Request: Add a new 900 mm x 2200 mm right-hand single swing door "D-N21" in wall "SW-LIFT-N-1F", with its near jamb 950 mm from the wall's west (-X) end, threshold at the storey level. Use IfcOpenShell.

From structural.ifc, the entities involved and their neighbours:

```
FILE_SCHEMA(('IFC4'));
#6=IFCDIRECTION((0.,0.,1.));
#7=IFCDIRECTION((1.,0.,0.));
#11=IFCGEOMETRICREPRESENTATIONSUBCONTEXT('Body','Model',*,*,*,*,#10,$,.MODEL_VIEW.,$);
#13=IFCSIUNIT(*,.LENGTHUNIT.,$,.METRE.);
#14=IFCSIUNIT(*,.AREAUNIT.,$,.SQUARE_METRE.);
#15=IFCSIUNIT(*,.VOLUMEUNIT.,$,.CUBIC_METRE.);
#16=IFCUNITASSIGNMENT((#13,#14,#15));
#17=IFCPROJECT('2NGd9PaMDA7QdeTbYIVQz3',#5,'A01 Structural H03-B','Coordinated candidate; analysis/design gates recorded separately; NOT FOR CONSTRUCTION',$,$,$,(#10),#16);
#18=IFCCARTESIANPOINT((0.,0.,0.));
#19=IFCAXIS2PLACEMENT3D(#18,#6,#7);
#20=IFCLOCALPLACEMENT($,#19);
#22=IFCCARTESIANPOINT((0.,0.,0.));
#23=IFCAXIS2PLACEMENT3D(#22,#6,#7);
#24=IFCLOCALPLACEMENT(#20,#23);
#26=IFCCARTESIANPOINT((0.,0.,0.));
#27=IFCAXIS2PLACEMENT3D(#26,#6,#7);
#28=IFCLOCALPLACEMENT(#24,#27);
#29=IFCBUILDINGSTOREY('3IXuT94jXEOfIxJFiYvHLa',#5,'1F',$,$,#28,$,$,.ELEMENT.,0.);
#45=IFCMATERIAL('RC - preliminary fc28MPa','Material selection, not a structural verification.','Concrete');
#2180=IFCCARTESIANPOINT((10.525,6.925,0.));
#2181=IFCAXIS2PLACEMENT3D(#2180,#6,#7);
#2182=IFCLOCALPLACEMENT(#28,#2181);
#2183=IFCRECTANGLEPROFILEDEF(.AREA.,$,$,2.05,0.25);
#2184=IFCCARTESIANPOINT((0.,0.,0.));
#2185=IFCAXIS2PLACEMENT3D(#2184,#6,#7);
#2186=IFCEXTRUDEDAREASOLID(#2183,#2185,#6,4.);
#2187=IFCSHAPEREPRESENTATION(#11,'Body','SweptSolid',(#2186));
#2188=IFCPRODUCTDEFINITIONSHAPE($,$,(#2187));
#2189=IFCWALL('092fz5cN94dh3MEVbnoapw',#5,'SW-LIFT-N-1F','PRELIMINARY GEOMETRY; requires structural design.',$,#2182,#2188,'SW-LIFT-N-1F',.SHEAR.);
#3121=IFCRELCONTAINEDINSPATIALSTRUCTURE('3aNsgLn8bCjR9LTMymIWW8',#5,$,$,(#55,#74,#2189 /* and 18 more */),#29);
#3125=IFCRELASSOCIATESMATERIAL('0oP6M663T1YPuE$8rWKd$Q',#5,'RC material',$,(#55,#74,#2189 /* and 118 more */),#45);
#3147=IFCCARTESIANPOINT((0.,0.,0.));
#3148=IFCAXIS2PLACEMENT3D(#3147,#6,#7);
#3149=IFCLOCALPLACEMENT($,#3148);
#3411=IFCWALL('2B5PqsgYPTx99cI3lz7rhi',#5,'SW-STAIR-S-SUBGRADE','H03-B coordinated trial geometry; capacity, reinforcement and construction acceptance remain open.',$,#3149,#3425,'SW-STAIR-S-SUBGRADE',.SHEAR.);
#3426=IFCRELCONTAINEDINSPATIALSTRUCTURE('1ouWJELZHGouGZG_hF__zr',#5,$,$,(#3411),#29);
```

```python
import numpy as np
import ifcopenshell
import ifcopenshell.api.feature
import ifcopenshell.api.geometry
import ifcopenshell.api.root
import ifcopenshell.api.spatial
import ifcopenshell.geom
import ifcopenshell.util.element
import ifcopenshell.util.placement
import ifcopenshell.util.representation
import ifcopenshell.util.shape
import ifcopenshell.util.unit

model = ifcopenshell.open("structural.ifc")
unit_scale = ifcopenshell.util.unit.calculate_unit_scale(model)
settings = ifcopenshell.geom.settings()


def volume(element):
    """Net volume in cubic metres, openings subtracted."""
    shape = ifcopenshell.geom.create_shape(settings, element)
    return ifcopenshell.util.shape.get_volume(shape.geometry)


wall = model.by_guid("092fz5cN94dh3MEVbnoapw")
storey = ifcopenshell.util.element.get_container(wall, ifc_class="IfcBuildingStorey")
context = ifcopenshell.util.representation.get_context(model, "Model", "Body", "MODEL_VIEW")
before = volume(wall)

width, height, from_end, sill = 0.9, 2.2, 0.95, 0.0  # metres

# The wall runs along its own X axis, and the end named is its -X end.
wall_shape = ifcopenshell.geom.create_shape(settings, wall)
x, y, z = ifcopenshell.util.shape.get_vertices(wall_shape.geometry).T
start = x.min() + from_end
face, thickness = float(y.min()), float(y.max() - y.min())
wall_matrix = ifcopenshell.util.placement.get_local_placement(wall.ObjectPlacement)
level = ifcopenshell.util.placement.get_local_placement(storey.ObjectPlacement)[2, 3]


def in_wall(x, y):
    """Placement at x, y metres in the wall's axes, at sill height."""
    matrix = wall_matrix.copy()
    matrix[:, 3] = wall_matrix @ np.array([x / unit_scale, y / unit_scale, 0.0, 1.0])
    matrix[2, 3] = level + sill / unit_scale
    return matrix


# Opening: a box that overshoots both wall faces by 50 mm.
opening = ifcopenshell.api.root.create_entity(model, ifc_class="IfcOpeningElement", predefined_type="OPENING")
box = ifcopenshell.api.geometry.add_wall_representation(
    model, context=context, length=width, height=height, thickness=thickness + 0.1
)
ifcopenshell.api.geometry.assign_representation(model, product=opening, representation=box)
ifcopenshell.api.geometry.edit_object_placement(model, product=opening, matrix=in_wall(start, face - 0.05), is_si=False)
ifcopenshell.api.feature.add_feature(model, feature=opening, element=wall)

door = ifcopenshell.api.root.create_entity(model, ifc_class="IfcDoor", name="D-N21", predefined_type="DOOR")
door.OverallWidth, door.OverallHeight = width / unit_scale, height / unit_scale
door.OperationType = "SINGLE_SWING_RIGHT"
body = ifcopenshell.api.geometry.add_door_representation(
    model,
    context=context,
    overall_width=door.OverallWidth,
    overall_height=door.OverallHeight,
    operation_type="SINGLE_SWING_RIGHT",
    lining_properties={"LiningDepth": thickness / unit_scale, "ThresholdDepth": thickness / unit_scale},
)
ifcopenshell.api.geometry.assign_representation(model, product=door, representation=body)
ifcopenshell.api.spatial.assign_container(model, products=[door], relating_structure=storey)
ifcopenshell.api.feature.add_filling(model, opening=opening, element=door)

# The lining spans the wall, so the door starts at the wall face.
ifcopenshell.api.geometry.edit_object_placement(model, product=door, matrix=in_wall(start, face), is_si=False)

after = volume(wall)

print(f"wall volume {before:.3f} -> {after:.3f} m3")

model.write("structural_edited.ifc")
```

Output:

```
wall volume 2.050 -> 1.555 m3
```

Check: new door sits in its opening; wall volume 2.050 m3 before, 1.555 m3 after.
